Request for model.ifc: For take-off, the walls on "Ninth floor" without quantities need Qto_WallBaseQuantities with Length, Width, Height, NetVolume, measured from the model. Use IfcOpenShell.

First a look at what the model holds.

```python
import ifcopenshell
import ifcopenshell.util.element
import ifcopenshell.util.unit

model = ifcopenshell.open("model.ifc")
print(model.schema)
for unit_type in ("LENGTHUNIT", "AREAUNIT", "VOLUMEUNIT"):
    print(unit_type, ifcopenshell.util.unit.calculate_unit_scale(model, unit_type))
storey = next(s for s in model.by_type("IfcBuildingStorey") if s.Name == "Ninth floor")
walls = [e for e in ifcopenshell.util.element.get_decomposition(storey) if e.is_a("IfcWall")]
for e in sorted(walls, key=lambda e: e.id()):
    print(e.id(), e.is_a(), e.Name, list(ifcopenshell.util.element.get_psets(e, qtos_only=True)), sep=" | ")
```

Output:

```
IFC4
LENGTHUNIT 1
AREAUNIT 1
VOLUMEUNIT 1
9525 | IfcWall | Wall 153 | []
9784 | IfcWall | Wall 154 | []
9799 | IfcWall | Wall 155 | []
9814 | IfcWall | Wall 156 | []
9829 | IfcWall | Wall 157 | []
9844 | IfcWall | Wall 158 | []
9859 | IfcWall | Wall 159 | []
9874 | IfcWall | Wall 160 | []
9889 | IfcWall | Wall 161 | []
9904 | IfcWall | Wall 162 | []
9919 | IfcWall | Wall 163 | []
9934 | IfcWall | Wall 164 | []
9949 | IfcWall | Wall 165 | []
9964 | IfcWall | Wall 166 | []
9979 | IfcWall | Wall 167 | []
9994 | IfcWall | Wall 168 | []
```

```python
import ifcopenshell
import ifcopenshell.api.pset
import ifcopenshell.geom
import ifcopenshell.util.element
import ifcopenshell.util.shape
import ifcopenshell.util.unit

model = ifcopenshell.open("model.ifc")
unit_scale = ifcopenshell.util.unit.calculate_unit_scale(model)
volume_scale = ifcopenshell.util.unit.calculate_unit_scale(model, "VOLUMEUNIT")
settings = ifcopenshell.geom.settings()

storey = next(s for s in model.by_type("IfcBuildingStorey") if s.Name == "Ninth floor")
walls = [e for e in ifcopenshell.util.element.get_decomposition(storey) if e.is_a("IfcWall")]

for e in sorted(walls, key=lambda e: e.id()):
    if ifcopenshell.util.element.get_psets(e, qtos_only=True, should_inherit=False):
        continue
    # Geometry comes back in metres, in the element's own axes.
    shape = ifcopenshell.geom.create_shape(settings, e)
    values = {
        "Length": ifcopenshell.util.shape.get_x(shape.geometry) / unit_scale,
        "Width": ifcopenshell.util.shape.get_y(shape.geometry) / unit_scale,
        "Height": ifcopenshell.util.shape.get_z(shape.geometry) / unit_scale,
        "NetVolume": ifcopenshell.util.shape.get_volume(shape.geometry) / volume_scale,
    }
    qto = ifcopenshell.api.pset.add_qto(model, product=e, name="Qto_WallBaseQuantities")
    ifcopenshell.api.pset.edit_qto(model, qto=qto, properties=values)
    print(e.id(), {k: round(v, 3) for k, v in values.items()})

model.write("model_rev.ifc")
```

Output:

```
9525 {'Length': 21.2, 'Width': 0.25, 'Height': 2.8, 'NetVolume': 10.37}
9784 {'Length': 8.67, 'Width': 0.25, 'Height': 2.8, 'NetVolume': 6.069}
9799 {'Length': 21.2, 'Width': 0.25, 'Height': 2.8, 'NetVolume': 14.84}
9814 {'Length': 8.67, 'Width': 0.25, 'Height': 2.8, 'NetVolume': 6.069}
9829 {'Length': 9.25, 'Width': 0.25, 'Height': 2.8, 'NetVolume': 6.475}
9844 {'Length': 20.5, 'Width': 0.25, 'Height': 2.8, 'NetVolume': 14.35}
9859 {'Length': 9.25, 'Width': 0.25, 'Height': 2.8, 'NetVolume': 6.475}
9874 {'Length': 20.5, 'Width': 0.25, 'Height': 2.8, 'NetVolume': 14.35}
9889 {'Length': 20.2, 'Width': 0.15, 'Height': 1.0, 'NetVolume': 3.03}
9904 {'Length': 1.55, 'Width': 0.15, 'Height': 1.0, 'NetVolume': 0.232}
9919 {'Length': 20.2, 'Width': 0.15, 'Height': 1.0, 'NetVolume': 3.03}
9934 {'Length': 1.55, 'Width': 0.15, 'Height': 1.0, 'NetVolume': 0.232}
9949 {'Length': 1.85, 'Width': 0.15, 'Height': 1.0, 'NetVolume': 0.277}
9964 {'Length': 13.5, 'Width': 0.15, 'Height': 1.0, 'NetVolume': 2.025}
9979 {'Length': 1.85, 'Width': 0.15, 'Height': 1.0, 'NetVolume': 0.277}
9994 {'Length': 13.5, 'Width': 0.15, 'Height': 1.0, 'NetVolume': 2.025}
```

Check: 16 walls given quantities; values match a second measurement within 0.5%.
